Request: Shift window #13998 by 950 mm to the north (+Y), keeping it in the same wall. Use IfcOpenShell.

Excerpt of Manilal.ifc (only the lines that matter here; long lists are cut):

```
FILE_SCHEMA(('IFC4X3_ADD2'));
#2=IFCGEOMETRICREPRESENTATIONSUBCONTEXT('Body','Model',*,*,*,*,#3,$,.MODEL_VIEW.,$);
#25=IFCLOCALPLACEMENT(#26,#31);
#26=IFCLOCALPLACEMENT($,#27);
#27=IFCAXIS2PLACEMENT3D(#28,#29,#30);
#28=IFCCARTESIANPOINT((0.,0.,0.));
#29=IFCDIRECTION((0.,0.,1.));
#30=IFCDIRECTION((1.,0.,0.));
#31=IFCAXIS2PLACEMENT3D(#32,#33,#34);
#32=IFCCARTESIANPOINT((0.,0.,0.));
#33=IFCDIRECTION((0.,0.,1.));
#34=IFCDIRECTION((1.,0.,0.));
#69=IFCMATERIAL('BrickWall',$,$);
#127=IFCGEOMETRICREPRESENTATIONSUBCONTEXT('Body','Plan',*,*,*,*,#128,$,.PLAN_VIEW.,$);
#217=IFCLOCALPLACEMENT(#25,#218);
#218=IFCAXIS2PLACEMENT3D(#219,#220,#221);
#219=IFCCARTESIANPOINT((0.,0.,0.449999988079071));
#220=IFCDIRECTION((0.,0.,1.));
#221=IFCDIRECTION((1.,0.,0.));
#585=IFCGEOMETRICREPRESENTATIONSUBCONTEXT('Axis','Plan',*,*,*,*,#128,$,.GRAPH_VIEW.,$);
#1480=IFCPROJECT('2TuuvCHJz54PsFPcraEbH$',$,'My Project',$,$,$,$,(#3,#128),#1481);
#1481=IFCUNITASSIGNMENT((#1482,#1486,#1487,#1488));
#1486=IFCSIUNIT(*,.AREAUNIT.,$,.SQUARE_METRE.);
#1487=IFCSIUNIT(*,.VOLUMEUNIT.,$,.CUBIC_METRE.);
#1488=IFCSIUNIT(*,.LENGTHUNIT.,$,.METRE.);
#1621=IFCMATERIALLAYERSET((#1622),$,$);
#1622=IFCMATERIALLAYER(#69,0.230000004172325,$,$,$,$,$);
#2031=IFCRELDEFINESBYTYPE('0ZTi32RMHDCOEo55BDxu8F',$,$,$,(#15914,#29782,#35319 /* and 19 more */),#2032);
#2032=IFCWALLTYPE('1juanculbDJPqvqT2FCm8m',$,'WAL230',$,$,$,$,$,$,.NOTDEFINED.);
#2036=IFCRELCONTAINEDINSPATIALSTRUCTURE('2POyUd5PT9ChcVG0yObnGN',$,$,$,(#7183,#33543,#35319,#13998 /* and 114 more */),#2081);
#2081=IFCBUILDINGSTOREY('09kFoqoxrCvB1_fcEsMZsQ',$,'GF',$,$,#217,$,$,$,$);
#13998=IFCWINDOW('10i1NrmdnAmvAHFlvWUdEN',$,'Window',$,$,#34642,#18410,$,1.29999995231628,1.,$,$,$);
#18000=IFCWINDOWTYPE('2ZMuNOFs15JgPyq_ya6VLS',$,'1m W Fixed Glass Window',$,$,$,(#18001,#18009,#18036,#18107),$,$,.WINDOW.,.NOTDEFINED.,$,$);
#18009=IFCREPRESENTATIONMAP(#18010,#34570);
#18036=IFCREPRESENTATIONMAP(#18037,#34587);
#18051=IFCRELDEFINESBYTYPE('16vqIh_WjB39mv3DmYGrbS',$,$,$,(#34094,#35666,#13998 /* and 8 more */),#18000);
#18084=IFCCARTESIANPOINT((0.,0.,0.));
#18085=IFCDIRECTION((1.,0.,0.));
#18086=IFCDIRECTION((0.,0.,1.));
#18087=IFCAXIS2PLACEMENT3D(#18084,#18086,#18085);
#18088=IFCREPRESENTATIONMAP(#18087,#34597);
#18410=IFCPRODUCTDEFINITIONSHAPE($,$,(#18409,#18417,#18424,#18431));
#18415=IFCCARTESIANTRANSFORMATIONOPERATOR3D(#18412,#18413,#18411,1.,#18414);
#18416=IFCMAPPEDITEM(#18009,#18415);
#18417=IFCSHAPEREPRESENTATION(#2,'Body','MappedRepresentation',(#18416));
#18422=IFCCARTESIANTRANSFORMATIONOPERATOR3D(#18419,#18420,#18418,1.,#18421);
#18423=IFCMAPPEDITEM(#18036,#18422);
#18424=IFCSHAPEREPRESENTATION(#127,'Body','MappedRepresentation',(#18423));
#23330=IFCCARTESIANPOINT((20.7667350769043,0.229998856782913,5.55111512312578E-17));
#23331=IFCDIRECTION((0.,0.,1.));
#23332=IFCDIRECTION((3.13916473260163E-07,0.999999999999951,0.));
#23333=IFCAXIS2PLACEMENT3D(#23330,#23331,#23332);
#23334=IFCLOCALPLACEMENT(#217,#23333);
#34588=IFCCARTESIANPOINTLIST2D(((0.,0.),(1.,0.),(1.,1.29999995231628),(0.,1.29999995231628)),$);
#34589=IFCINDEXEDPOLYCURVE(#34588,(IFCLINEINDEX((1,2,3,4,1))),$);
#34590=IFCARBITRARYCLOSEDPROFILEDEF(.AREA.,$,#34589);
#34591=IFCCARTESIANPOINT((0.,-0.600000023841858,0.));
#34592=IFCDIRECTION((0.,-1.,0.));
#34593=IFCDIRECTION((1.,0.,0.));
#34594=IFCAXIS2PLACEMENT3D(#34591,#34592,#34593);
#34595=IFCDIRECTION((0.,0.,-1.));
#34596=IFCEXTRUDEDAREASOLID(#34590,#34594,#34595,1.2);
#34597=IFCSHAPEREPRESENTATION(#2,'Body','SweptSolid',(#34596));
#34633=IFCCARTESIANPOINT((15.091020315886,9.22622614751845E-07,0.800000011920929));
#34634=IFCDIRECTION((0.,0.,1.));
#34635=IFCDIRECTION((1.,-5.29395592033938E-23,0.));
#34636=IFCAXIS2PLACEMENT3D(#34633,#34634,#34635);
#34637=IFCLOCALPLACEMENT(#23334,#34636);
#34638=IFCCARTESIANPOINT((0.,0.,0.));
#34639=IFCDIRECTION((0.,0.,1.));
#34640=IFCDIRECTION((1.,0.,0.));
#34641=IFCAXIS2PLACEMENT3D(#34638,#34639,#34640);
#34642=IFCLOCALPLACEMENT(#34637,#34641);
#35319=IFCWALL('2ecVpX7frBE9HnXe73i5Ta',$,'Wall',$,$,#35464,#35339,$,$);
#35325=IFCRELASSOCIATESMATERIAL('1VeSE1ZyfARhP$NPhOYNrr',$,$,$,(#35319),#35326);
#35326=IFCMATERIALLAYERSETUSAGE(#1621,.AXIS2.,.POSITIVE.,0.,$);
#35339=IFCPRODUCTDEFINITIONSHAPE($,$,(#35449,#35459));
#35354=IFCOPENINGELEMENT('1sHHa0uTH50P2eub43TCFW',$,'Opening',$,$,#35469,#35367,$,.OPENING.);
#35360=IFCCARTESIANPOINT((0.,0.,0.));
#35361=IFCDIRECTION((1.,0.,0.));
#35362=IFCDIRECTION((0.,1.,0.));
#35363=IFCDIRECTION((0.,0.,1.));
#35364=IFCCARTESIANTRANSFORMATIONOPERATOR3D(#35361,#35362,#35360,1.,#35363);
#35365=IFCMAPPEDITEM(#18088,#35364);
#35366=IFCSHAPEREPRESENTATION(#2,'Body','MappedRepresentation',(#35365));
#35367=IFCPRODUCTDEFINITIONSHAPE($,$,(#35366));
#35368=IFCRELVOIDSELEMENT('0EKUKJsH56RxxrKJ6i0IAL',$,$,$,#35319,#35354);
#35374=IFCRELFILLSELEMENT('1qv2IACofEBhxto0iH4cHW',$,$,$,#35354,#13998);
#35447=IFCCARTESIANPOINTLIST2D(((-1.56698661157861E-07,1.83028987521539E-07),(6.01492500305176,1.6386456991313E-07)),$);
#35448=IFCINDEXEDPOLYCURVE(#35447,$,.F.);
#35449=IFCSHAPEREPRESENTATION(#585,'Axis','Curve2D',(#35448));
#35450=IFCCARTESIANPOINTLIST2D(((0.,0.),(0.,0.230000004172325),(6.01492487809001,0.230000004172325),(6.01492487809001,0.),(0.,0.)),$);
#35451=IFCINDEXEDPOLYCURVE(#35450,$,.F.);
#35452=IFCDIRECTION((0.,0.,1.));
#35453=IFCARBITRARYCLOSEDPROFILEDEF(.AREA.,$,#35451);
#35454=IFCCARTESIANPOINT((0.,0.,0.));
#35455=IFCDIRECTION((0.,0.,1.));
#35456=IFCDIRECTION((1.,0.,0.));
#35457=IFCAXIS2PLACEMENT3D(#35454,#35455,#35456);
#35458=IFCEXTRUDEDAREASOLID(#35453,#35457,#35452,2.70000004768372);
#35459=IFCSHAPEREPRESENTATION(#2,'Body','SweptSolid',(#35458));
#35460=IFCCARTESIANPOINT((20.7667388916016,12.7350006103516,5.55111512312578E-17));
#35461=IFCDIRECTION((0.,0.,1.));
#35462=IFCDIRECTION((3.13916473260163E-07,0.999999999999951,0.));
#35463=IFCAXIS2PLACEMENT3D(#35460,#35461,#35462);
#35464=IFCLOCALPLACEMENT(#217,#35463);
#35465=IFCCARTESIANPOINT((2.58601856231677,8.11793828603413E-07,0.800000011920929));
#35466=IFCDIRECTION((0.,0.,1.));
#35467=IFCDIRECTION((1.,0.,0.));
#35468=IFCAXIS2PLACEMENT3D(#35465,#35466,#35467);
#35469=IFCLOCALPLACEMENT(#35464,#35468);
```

```python
import ifcopenshell
import ifcopenshell.api.geometry
import ifcopenshell.util.placement

model = ifcopenshell.open("Manilal.ifc")

window = model.by_guid("10i1NrmdnAmvAHFlvWUdEN")
opening = window.FillsVoids[0].RelatingOpeningElement
wall = opening.VoidsElements[0].RelatingBuildingElement

wall_matrix = ifcopenshell.util.placement.get_local_placement(wall.ObjectPlacement)
shift = wall_matrix[:3, 0] * 0.95
before = ifcopenshell.util.placement.get_local_placement(window.ObjectPlacement)[:3, 3].copy()

# The window is not placed relative to its opening, so move both.
for product in (opening, window):
    matrix = ifcopenshell.util.placement.get_local_placement(product.ObjectPlacement)
    matrix[:3, 3] += shift
    ifcopenshell.api.geometry.edit_object_placement(model, product=product, matrix=matrix, is_si=False)

after = ifcopenshell.util.placement.get_local_placement(window.ObjectPlacement)[:3, 3]
print("window moved by", (after - before).round(3) + 0.0)

model.write("Manilal_v2.ifc")
```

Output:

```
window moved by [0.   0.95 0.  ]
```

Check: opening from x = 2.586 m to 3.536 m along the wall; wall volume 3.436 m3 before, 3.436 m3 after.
